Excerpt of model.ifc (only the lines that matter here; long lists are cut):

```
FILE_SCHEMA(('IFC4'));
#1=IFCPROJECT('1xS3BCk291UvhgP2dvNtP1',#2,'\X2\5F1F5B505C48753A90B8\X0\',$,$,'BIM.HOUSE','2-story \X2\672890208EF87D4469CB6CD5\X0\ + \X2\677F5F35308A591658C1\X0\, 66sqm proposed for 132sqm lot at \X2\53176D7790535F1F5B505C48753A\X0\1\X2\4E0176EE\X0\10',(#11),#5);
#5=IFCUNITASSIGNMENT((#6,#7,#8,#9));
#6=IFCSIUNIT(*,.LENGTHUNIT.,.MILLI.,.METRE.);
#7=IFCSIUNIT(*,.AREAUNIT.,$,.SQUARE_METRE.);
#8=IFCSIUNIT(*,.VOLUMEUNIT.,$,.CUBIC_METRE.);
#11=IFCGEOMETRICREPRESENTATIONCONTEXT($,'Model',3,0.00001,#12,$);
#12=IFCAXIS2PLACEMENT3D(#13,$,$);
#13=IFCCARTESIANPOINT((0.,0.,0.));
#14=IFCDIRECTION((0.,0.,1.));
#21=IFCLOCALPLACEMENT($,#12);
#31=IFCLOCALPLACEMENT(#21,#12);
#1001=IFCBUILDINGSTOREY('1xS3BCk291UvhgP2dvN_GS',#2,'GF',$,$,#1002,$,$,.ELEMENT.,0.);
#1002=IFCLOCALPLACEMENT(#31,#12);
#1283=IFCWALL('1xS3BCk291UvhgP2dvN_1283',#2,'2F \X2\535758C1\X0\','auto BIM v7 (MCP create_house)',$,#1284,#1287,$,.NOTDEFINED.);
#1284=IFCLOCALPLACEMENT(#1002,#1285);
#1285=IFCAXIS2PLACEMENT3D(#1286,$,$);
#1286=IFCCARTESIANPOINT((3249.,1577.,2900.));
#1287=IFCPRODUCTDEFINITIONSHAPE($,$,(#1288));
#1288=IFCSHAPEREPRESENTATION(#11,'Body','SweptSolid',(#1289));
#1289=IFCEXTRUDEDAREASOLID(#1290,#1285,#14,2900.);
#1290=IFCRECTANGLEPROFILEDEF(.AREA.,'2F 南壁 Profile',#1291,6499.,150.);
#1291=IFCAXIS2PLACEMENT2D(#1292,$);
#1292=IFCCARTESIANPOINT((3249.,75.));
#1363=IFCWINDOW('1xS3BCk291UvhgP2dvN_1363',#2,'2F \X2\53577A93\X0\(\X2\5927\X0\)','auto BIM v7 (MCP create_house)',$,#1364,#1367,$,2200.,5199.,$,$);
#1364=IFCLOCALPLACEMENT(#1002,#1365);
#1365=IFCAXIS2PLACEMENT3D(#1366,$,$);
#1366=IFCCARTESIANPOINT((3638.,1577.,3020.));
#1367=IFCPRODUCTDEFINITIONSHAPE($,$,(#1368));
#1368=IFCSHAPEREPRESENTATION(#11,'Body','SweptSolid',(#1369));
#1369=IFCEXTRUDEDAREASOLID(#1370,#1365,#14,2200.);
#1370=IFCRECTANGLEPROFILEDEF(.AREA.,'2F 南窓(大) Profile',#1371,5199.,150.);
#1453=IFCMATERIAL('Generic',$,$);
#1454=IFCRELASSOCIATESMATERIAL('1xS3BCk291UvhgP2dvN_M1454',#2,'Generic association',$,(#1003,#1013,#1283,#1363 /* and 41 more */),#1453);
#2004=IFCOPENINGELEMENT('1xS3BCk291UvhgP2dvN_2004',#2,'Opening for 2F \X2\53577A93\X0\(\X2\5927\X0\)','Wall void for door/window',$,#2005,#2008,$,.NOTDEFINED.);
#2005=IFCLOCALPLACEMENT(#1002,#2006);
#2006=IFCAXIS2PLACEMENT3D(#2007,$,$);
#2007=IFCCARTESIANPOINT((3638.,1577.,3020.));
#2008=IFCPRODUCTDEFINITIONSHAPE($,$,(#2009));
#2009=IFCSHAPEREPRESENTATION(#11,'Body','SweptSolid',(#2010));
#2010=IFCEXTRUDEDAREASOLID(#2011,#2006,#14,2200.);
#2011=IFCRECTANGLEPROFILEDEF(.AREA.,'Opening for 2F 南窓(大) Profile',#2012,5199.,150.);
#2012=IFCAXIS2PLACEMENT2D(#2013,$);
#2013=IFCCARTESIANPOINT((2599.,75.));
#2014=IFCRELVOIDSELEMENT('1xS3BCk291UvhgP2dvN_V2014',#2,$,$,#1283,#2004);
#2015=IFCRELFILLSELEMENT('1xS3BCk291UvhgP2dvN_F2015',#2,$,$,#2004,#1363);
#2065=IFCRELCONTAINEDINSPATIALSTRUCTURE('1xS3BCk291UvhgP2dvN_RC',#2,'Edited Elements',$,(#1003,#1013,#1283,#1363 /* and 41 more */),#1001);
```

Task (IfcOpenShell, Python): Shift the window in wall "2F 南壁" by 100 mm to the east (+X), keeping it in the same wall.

```python
import ifcopenshell
import ifcopenshell.api.geometry
import ifcopenshell.util.placement
import ifcopenshell.util.unit

model = ifcopenshell.open("model.ifc")
unit_scale = ifcopenshell.util.unit.calculate_unit_scale(model)

window = model.by_guid("1xS3BCk291UvhgP2dvN_1363")
opening = window.FillsVoids[0].RelatingOpeningElement
wall = opening.VoidsElements[0].RelatingBuildingElement

wall_matrix = ifcopenshell.util.placement.get_local_placement(wall.ObjectPlacement)
shift = wall_matrix[:3, 0] * 0.1 / unit_scale
before = ifcopenshell.util.placement.get_local_placement(window.ObjectPlacement)[:3, 3].copy()

# The window is not placed relative to its opening, so move both.
for product in (opening, window):
    matrix = ifcopenshell.util.placement.get_local_placement(product.ObjectPlacement)
    matrix[:3, 3] += shift
    ifcopenshell.api.geometry.edit_object_placement(model, product=product, matrix=matrix, is_si=False)

after = ifcopenshell.util.placement.get_local_placement(window.ObjectPlacement)[:3, 3]
print("window moved by", (after - before).round(3) + 0.0)

model.write("model_updated.ifc")
```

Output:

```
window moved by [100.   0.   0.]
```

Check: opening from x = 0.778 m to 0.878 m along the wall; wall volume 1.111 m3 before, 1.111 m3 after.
